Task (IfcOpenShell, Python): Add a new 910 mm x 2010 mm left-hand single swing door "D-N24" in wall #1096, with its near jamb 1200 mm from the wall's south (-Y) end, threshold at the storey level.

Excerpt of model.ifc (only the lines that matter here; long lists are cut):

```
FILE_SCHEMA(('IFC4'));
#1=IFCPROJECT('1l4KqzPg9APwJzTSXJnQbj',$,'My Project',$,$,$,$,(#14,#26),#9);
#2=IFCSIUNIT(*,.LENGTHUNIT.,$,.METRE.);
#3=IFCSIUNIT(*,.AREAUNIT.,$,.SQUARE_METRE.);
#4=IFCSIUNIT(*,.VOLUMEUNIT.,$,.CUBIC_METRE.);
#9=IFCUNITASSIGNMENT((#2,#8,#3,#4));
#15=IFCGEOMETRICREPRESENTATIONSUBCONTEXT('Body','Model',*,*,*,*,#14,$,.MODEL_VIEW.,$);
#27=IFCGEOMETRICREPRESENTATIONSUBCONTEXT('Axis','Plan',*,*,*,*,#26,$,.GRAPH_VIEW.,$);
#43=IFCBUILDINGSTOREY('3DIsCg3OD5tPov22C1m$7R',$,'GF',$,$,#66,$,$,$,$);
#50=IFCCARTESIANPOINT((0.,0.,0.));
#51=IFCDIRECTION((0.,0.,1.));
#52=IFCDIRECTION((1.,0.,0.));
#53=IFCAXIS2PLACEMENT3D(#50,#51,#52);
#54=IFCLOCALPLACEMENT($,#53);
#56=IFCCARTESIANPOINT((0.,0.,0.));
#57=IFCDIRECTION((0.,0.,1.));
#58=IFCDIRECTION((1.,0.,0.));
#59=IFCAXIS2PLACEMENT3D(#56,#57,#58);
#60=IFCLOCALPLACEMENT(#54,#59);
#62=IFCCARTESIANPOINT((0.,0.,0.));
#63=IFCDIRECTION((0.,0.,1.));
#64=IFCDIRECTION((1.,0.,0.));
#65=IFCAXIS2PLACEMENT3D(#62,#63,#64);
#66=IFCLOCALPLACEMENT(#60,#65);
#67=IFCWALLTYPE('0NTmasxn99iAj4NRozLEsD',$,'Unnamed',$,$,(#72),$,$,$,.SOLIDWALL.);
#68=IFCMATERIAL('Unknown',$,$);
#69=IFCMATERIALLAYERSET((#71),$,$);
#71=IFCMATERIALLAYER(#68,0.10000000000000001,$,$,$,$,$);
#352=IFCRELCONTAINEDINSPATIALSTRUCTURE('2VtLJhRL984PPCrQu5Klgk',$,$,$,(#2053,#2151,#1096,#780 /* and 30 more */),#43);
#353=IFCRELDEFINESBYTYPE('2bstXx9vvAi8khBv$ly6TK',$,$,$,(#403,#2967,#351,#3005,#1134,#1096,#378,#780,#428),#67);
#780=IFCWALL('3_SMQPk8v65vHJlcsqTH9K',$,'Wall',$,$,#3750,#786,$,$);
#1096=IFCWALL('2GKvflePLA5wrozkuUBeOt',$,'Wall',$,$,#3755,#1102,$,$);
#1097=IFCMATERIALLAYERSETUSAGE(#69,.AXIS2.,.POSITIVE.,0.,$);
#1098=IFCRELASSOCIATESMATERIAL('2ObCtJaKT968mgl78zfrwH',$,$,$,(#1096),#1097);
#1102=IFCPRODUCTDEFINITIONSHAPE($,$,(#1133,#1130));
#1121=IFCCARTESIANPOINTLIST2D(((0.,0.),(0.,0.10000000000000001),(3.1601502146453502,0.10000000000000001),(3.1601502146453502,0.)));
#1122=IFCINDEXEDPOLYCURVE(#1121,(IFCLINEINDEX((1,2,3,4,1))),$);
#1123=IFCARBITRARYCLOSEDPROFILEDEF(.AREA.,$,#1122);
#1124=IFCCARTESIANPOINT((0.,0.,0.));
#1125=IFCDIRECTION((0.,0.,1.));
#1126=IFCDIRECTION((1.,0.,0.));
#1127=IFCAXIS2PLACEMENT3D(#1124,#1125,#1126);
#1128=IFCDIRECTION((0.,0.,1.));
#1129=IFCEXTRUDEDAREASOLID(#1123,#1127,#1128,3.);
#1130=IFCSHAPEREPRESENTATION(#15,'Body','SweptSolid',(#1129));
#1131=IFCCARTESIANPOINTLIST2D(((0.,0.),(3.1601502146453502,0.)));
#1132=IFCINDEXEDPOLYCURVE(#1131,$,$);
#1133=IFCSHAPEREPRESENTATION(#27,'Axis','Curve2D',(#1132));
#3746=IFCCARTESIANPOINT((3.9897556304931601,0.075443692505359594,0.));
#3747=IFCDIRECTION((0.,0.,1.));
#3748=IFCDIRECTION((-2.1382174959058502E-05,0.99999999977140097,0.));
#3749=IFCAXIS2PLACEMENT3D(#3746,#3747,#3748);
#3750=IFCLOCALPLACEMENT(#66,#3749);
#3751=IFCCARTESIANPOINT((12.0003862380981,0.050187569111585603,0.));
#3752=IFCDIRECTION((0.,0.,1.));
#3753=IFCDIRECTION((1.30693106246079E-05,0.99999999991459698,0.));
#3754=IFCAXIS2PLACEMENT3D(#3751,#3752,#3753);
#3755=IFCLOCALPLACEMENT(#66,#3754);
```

```python
import numpy as np
import ifcopenshell
import ifcopenshell.api.feature
import ifcopenshell.api.geometry
import ifcopenshell.api.root
import ifcopenshell.api.spatial
import ifcopenshell.geom
import ifcopenshell.util.element
import ifcopenshell.util.placement
import ifcopenshell.util.representation
import ifcopenshell.util.shape
import ifcopenshell.util.unit

model = ifcopenshell.open("model.ifc")
unit_scale = ifcopenshell.util.unit.calculate_unit_scale(model)
settings = ifcopenshell.geom.settings()


def volume(element):
    """Net volume in cubic metres, openings subtracted."""
    shape = ifcopenshell.geom.create_shape(settings, element)
    return ifcopenshell.util.shape.get_volume(shape.geometry)


wall = model.by_id(1096)
storey = ifcopenshell.util.element.get_container(wall, ifc_class="IfcBuildingStorey")
context = ifcopenshell.util.representation.get_context(model, "Model", "Body", "MODEL_VIEW")
before = volume(wall)

width, height, from_end, sill = 0.91, 2.01, 1.2, 0.0  # metres

# The wall runs along its own X axis, and the end named is its -X end.
wall_shape = ifcopenshell.geom.create_shape(settings, wall)
x, y, z = ifcopenshell.util.shape.get_vertices(wall_shape.geometry).T
start = x.min() + from_end
face, thickness = float(y.min()), float(y.max() - y.min())
wall_matrix = ifcopenshell.util.placement.get_local_placement(wall.ObjectPlacement)
level = ifcopenshell.util.placement.get_local_placement(storey.ObjectPlacement)[2, 3]


def in_wall(x, y):
    """Placement at x, y metres in the wall's axes, at sill height."""
    matrix = wall_matrix.copy()
    matrix[:, 3] = wall_matrix @ np.array([x / unit_scale, y / unit_scale, 0.0, 1.0])
    matrix[2, 3] = level + sill / unit_scale
    return matrix


# Opening: a box that overshoots both wall faces by 50 mm.
opening = ifcopenshell.api.root.create_entity(model, ifc_class="IfcOpeningElement", predefined_type="OPENING")
box = ifcopenshell.api.geometry.add_wall_representation(
    model, context=context, length=width, height=height, thickness=thickness + 0.1
)
ifcopenshell.api.geometry.assign_representation(model, product=opening, representation=box)
ifcopenshell.api.geometry.edit_object_placement(model, product=opening, matrix=in_wall(start, face - 0.05), is_si=False)
ifcopenshell.api.feature.add_feature(model, feature=opening, element=wall)

door = ifcopenshell.api.root.create_entity(model, ifc_class="IfcDoor", name="D-N24", predefined_type="DOOR")
door.OverallWidth, door.OverallHeight = width / unit_scale, height / unit_scale
door.OperationType = "SINGLE_SWING_LEFT"
body = ifcopenshell.api.geometry.add_door_representation(
    model,
    context=context,
    overall_width=door.OverallWidth,
    overall_height=door.OverallHeight,
    operation_type="SINGLE_SWING_LEFT",
    lining_properties={"LiningDepth": thickness / unit_scale, "ThresholdDepth": thickness / unit_scale},
)
ifcopenshell.api.geometry.assign_representation(model, product=door, representation=body)
ifcopenshell.api.spatial.assign_container(model, products=[door], relating_structure=storey)
ifcopenshell.api.feature.add_filling(model, opening=opening, element=door)

# The lining spans the wall, so the door starts at the wall face.
ifcopenshell.api.geometry.edit_object_placement(model, product=door, matrix=in_wall(start, face), is_si=False)

after = volume(wall)

print(f"wall volume {before:.3f} -> {after:.3f} m3")

model.write("model_rev.ifc")
```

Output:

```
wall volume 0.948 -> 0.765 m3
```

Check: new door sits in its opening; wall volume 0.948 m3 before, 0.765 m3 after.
